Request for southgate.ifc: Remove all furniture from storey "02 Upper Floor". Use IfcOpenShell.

First a look at what the model holds.

```python
import ifcopenshell
import ifcopenshell.util.element

model = ifcopenshell.open("southgate.ifc")
print(model.schema)
storey = next(s for s in model.by_type("IfcBuildingStorey") if s.Name == "02 Upper Floor")
furniture = [e for e in ifcopenshell.util.element.get_decomposition(storey) if e.is_a("IfcFurnishingElement")]
seen = {}
for e in furniture:
    element_type = ifcopenshell.util.element.get_type(e)
    name = element_type.Name if element_type not in (None, e) else None
    seen[name] = seen.get(name, 0) + 1
for name, count in sorted(seen.items(), key=str):
    print(count, "x", name)
```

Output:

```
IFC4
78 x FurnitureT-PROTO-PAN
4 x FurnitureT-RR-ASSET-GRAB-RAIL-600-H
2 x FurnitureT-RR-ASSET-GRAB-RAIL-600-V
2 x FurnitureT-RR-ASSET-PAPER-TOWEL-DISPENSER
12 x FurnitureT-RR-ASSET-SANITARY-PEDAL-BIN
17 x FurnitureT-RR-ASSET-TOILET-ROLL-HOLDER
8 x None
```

```python
import ifcopenshell
import ifcopenshell.api.root
import ifcopenshell.util.element

model = ifcopenshell.open("southgate.ifc")

storey = next(s for s in model.by_type("IfcBuildingStorey") if s.Name == "02 Upper Floor")
furniture = [e for e in ifcopenshell.util.element.get_decomposition(storey) if e.is_a("IfcFurnishingElement")]

for e in furniture:
    ifcopenshell.api.root.remove_product(model, product=e)
print(len(furniture), "removed")

model.write("southgate_updated.ifc")
```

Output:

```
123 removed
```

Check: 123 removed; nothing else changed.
